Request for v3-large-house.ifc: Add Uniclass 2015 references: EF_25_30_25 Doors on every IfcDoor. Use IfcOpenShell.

First a look at what the model holds.

```python
import ifcopenshell

model = ifcopenshell.open("v3-large-house.ifc")
print(model.schema)
print("classifications:", [c.Name for c in model.by_type("IfcClassification")])
for ifc_class in ("IfcDoor", "IfcRoof", "IfcStair", "IfcWall", "IfcWindow"):
    print(ifc_class, len(model.by_type(ifc_class)))
```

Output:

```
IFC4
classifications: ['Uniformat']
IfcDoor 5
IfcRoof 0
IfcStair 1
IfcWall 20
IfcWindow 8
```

```python
import ifcopenshell
import ifcopenshell.api.classification

model = ifcopenshell.open("v3-large-house.ifc")

system = ifcopenshell.api.classification.add_classification(model, classification="Uniclass 2015")

codes = {
    "IfcDoor": ("EF_25_30_25", "Doors"),
}
for ifc_class, (code, name) in codes.items():
    products = model.by_type(ifc_class)
    ifcopenshell.api.classification.add_reference(
        model, products=products, classification=system, identification=code, name=name
    )
    print(code, len(products))

model.write("v3-large-house_rev.ifc")
```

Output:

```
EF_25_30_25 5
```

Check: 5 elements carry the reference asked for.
